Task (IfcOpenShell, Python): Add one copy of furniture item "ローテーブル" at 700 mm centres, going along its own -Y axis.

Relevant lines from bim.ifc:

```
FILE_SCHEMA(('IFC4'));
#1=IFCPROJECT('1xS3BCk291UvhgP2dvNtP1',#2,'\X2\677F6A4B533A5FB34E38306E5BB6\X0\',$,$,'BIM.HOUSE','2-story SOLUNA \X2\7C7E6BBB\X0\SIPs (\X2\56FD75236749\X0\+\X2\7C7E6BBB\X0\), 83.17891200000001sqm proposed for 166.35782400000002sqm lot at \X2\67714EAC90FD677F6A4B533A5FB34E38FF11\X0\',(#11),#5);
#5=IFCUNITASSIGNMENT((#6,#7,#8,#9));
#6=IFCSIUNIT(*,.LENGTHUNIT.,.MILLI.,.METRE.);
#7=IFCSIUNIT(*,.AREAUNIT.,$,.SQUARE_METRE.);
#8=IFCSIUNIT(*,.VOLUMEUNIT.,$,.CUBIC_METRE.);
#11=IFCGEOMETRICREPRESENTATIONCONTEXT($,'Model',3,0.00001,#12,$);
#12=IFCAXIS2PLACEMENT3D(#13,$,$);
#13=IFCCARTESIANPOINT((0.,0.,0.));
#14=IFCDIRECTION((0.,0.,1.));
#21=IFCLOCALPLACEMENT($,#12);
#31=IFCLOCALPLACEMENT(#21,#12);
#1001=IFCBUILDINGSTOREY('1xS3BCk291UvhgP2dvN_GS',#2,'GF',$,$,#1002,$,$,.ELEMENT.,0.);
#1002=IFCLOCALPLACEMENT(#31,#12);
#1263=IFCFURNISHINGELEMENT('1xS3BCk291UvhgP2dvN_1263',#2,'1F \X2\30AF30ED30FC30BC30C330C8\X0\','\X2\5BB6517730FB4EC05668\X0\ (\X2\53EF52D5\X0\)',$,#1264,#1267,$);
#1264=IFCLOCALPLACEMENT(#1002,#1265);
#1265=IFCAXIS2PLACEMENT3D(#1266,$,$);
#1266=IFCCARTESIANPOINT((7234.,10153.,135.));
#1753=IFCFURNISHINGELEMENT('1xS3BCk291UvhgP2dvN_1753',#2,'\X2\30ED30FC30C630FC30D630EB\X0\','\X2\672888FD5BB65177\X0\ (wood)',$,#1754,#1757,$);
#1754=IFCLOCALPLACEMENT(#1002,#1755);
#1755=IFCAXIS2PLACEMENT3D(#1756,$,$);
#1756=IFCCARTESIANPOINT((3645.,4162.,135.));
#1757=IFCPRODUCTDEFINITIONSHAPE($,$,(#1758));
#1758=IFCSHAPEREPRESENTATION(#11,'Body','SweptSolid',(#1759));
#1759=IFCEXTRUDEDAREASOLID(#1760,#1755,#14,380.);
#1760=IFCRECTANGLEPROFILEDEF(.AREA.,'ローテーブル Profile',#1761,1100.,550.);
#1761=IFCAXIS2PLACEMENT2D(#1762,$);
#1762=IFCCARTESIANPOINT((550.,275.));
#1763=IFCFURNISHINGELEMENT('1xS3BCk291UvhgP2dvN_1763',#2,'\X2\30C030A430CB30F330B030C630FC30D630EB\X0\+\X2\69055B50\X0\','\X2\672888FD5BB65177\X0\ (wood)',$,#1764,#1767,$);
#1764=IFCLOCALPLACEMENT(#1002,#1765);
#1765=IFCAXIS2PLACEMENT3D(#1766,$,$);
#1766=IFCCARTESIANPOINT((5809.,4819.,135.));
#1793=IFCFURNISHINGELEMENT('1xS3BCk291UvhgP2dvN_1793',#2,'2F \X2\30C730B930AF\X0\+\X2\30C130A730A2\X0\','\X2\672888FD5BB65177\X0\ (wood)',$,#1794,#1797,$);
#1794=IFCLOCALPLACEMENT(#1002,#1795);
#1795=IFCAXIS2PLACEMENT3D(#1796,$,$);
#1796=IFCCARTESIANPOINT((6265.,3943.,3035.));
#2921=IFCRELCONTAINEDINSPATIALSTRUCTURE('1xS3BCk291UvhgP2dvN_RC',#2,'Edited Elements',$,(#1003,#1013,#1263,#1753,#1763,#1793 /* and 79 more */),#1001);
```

```python
import ifcopenshell
import ifcopenshell.api.geometry
import ifcopenshell.api.root
import ifcopenshell.util.element
import ifcopenshell.util.placement
import ifcopenshell.util.unit

model = ifcopenshell.open("bim.ifc")
unit_scale = ifcopenshell.util.unit.calculate_unit_scale(model)


def reuse_history(source, copy):
    """copy_class also copies each property set's owner history, people and application; keep the originals."""
    for rel in copy.IsDefinedBy:
        if rel.is_a("IfcRelDefinesByProperties") and (history := rel.RelatingPropertyDefinition.OwnerHistory):
            rel.RelatingPropertyDefinition.OwnerHistory = source.OwnerHistory
            ifcopenshell.util.element.remove_deep2(model, history)


source = model.by_guid("1xS3BCk291UvhgP2dvN_1753")
base = ifcopenshell.util.placement.get_local_placement(source.ObjectPlacement)
step = -base[:3, 1] * 0.7 / unit_scale

for i in range(1, 2):
    copy = ifcopenshell.api.root.copy_class(model, product=source)
    copy.Representation = ifcopenshell.util.element.copy_deep(
        model, source.Representation, exclude=["IfcGeometricRepresentationContext", "IfcRepresentationMap"]
    )
    reuse_history(source, copy)
    matrix = base.copy()
    matrix[:3, 3] += i * step
    print("added at", matrix[:3, 3].round(3) + 0.0)
    ifcopenshell.api.geometry.edit_object_placement(model, product=copy, matrix=matrix, is_si=False)

model.write("bim_v2.ifc")
```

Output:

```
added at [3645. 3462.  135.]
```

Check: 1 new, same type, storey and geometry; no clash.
